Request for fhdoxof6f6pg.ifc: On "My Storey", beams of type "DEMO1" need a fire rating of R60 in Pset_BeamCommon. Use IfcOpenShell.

First a look at what the model holds.

```python
import ifcopenshell
import ifcopenshell.util.element

model = ifcopenshell.open("fhdoxof6f6pg.ifc")
print(model.schema)
storey = next(s for s in model.by_type("IfcBuildingStorey") if s.Name == "My Storey")
beams = [e for e in ifcopenshell.util.element.get_decomposition(storey) if e.is_a("IfcBeam")]
seen = {}
for e in beams:
    element_type = ifcopenshell.util.element.get_type(e)
    key = (element_type.Name if element_type != e and element_type else None, ifcopenshell.util.element.get_pset(e, "Pset_BeamCommon", "FireRating"))
    seen[key] = seen.get(key, 0) + 1
for (name, value), count in sorted(seen.items(), key=str):
    print(count, "x", name, "|", value)
```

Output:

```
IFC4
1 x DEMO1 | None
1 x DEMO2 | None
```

```python
import ifcopenshell
import ifcopenshell.api.pset
import ifcopenshell.util.element

model = ifcopenshell.open("fhdoxof6f6pg.ifc")

storey = next(s for s in model.by_type("IfcBuildingStorey") if s.Name == "My Storey")
beams = [e for e in ifcopenshell.util.element.get_decomposition(storey) if e.is_a("IfcBeam")]

count = 0
for e in beams:
    element_type = ifcopenshell.util.element.get_type(e)
    if element_type in (None, e) or element_type.Name != "DEMO1":
        continue
    # add_pset returns the element's existing set when there is one.
    pset = ifcopenshell.api.pset.add_pset(model, product=e, name="Pset_BeamCommon")
    ifcopenshell.api.pset.edit_pset(model, pset=pset, properties={"FireRating": "R60"})
    count += 1

print(count, "beams updated")

model.write("fhdoxof6f6pg_rev.ifc")
```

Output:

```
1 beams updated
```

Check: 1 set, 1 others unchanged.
